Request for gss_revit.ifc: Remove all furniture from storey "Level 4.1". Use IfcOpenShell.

First a look at what the model holds.

```python
import ifcopenshell
import ifcopenshell.util.element

model = ifcopenshell.open("gss_revit.ifc")
print(model.schema)
storey = next(s for s in model.by_type("IfcBuildingStorey") if s.Name == "Level 4.1")
furniture = [e for e in ifcopenshell.util.element.get_decomposition(storey) if e.is_a("IfcFurnishingElement")]
seen = {}
for e in furniture:
    element_type = ifcopenshell.util.element.get_type(e)
    name = element_type.Name if element_type not in (None, e) else None
    seen[name] = seen.get(name, 0) + 1
for name, count in sorted(seen.items(), key=str):
    print(count, "x", name)
```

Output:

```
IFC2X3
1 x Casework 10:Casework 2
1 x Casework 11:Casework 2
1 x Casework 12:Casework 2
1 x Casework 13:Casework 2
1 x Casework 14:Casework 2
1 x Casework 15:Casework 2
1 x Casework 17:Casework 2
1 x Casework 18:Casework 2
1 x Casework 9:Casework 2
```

```python
import ifcopenshell
import ifcopenshell.api.root
import ifcopenshell.util.element

model = ifcopenshell.open("gss_revit.ifc")

storey = next(s for s in model.by_type("IfcBuildingStorey") if s.Name == "Level 4.1")
furniture = [e for e in ifcopenshell.util.element.get_decomposition(storey) if e.is_a("IfcFurnishingElement")]

for e in furniture:
    ifcopenshell.api.root.remove_product(model, product=e)
print(len(furniture), "removed")

model.write("gss_revit_edited.ifc")
```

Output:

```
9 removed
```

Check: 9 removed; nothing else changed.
